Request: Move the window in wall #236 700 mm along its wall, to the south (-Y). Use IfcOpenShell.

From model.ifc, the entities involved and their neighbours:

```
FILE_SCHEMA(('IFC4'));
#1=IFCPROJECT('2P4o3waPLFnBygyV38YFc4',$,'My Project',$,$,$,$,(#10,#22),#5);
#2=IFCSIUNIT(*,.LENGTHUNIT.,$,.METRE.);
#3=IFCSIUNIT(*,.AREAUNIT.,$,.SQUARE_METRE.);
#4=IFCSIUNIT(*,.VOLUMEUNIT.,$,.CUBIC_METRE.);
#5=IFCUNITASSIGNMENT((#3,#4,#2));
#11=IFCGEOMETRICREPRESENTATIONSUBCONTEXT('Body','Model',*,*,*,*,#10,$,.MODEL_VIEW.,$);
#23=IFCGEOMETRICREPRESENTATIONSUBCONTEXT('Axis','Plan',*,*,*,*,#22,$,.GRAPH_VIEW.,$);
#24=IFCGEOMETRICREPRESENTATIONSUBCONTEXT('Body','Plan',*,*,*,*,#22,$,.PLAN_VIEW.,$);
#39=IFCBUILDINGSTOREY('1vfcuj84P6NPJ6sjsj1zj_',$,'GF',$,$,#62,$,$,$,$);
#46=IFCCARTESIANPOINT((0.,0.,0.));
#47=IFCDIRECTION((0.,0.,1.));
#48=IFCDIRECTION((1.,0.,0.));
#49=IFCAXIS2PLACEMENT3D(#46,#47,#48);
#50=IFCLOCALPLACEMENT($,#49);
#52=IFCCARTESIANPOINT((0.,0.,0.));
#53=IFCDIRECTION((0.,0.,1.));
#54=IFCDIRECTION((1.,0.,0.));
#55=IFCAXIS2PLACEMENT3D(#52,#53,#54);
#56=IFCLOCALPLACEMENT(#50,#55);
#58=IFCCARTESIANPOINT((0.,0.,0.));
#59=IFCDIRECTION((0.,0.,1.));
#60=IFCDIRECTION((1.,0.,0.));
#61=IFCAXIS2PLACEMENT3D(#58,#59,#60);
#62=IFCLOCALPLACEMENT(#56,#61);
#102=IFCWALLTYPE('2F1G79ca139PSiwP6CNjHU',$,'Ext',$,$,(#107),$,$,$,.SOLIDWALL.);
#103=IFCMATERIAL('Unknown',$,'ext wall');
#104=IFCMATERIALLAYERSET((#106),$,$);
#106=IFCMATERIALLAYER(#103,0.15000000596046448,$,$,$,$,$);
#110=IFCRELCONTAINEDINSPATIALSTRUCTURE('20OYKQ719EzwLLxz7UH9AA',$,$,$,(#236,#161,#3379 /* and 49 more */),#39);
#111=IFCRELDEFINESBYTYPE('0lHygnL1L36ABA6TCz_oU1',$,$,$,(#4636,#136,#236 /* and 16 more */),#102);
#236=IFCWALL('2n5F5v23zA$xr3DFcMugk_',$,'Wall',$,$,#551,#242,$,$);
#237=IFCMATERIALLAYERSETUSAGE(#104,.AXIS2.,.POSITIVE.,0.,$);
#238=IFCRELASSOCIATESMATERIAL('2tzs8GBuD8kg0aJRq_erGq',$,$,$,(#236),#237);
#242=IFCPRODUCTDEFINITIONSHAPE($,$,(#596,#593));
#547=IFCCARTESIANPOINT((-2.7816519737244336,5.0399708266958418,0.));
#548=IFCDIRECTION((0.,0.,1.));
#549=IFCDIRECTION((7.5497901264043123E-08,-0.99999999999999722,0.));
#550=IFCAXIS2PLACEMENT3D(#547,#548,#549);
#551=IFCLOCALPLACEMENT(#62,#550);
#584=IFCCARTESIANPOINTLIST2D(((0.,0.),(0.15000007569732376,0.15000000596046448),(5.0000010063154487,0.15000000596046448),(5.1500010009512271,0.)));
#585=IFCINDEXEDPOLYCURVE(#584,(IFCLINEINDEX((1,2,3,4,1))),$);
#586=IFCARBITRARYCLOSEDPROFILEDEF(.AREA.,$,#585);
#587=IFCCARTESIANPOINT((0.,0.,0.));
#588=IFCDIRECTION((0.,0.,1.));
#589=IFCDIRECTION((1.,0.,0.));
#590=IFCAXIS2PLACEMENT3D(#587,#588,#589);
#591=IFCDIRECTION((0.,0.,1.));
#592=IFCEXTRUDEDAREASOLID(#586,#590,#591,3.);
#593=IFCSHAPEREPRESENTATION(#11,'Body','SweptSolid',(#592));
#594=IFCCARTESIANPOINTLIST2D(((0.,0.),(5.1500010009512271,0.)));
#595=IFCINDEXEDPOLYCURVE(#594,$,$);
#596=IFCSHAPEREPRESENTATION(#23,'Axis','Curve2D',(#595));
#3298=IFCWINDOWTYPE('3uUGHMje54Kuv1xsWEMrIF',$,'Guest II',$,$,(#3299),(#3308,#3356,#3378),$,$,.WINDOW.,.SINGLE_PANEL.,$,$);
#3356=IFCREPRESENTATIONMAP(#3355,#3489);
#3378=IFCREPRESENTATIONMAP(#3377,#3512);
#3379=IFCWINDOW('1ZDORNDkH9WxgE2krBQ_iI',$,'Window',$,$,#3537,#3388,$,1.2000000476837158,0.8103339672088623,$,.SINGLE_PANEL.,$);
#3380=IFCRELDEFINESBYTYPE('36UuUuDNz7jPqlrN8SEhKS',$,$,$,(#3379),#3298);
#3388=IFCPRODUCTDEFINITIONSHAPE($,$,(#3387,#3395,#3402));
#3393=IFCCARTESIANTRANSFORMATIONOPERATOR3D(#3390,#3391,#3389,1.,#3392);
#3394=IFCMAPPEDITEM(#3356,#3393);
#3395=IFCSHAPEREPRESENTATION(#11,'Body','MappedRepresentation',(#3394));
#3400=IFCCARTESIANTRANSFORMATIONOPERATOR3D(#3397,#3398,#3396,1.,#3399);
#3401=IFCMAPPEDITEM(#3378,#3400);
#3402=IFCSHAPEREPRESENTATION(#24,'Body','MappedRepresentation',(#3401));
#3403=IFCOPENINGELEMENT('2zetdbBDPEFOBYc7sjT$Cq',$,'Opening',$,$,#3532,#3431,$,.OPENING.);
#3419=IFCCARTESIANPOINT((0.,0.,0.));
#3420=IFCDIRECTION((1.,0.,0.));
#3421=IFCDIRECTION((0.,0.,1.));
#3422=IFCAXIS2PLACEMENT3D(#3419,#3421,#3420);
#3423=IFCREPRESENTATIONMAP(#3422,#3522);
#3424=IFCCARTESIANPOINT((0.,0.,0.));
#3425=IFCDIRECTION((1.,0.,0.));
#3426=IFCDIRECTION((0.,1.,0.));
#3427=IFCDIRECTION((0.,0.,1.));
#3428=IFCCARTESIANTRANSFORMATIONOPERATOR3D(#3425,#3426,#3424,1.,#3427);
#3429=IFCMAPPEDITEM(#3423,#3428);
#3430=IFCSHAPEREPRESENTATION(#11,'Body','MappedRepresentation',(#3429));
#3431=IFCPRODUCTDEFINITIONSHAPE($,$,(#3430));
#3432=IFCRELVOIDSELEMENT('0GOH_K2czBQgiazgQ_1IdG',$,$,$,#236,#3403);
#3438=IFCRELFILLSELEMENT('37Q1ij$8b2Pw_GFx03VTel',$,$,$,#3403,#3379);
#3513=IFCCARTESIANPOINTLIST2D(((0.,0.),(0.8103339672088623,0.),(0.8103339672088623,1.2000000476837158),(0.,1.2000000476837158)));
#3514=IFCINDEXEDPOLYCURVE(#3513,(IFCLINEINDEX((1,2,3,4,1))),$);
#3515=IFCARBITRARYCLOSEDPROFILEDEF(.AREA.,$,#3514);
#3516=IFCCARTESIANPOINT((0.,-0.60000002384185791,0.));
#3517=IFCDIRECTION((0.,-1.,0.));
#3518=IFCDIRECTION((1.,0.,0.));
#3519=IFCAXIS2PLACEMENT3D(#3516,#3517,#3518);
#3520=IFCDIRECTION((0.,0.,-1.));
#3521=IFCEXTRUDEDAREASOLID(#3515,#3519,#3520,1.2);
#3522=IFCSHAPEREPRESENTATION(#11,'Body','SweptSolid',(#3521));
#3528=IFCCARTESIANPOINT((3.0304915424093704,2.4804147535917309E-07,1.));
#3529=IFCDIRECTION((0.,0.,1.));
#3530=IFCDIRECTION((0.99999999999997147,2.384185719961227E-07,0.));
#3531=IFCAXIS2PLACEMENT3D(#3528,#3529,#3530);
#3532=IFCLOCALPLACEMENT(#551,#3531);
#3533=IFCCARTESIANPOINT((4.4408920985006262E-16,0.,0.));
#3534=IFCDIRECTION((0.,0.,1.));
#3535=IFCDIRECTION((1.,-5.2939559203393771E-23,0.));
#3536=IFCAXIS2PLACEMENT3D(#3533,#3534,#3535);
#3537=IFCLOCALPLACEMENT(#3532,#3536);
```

```python
import ifcopenshell
import ifcopenshell.api.geometry
import ifcopenshell.util.placement

model = ifcopenshell.open("model.ifc")

window = model.by_guid("1ZDORNDkH9WxgE2krBQ_iI")
opening = window.FillsVoids[0].RelatingOpeningElement
wall = opening.VoidsElements[0].RelatingBuildingElement

wall_matrix = ifcopenshell.util.placement.get_local_placement(wall.ObjectPlacement)
shift = wall_matrix[:3, 0] * 0.7
before = ifcopenshell.util.placement.get_local_placement(window.ObjectPlacement)[:3, 3].copy()

# The window is placed relative to its opening, so it follows when the opening moves.
matrix = ifcopenshell.util.placement.get_local_placement(opening.ObjectPlacement)
matrix[:3, 3] += shift
ifcopenshell.api.geometry.edit_object_placement(
    model, product=opening, matrix=matrix, is_si=False, should_transform_children=True
)

after = ifcopenshell.util.placement.get_local_placement(window.ObjectPlacement)[:3, 3]
print("window moved by", (after - before).round(3) + 0.0)

model.write("model-out.ifc")
```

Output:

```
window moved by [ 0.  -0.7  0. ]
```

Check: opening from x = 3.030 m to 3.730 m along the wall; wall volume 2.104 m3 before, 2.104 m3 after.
